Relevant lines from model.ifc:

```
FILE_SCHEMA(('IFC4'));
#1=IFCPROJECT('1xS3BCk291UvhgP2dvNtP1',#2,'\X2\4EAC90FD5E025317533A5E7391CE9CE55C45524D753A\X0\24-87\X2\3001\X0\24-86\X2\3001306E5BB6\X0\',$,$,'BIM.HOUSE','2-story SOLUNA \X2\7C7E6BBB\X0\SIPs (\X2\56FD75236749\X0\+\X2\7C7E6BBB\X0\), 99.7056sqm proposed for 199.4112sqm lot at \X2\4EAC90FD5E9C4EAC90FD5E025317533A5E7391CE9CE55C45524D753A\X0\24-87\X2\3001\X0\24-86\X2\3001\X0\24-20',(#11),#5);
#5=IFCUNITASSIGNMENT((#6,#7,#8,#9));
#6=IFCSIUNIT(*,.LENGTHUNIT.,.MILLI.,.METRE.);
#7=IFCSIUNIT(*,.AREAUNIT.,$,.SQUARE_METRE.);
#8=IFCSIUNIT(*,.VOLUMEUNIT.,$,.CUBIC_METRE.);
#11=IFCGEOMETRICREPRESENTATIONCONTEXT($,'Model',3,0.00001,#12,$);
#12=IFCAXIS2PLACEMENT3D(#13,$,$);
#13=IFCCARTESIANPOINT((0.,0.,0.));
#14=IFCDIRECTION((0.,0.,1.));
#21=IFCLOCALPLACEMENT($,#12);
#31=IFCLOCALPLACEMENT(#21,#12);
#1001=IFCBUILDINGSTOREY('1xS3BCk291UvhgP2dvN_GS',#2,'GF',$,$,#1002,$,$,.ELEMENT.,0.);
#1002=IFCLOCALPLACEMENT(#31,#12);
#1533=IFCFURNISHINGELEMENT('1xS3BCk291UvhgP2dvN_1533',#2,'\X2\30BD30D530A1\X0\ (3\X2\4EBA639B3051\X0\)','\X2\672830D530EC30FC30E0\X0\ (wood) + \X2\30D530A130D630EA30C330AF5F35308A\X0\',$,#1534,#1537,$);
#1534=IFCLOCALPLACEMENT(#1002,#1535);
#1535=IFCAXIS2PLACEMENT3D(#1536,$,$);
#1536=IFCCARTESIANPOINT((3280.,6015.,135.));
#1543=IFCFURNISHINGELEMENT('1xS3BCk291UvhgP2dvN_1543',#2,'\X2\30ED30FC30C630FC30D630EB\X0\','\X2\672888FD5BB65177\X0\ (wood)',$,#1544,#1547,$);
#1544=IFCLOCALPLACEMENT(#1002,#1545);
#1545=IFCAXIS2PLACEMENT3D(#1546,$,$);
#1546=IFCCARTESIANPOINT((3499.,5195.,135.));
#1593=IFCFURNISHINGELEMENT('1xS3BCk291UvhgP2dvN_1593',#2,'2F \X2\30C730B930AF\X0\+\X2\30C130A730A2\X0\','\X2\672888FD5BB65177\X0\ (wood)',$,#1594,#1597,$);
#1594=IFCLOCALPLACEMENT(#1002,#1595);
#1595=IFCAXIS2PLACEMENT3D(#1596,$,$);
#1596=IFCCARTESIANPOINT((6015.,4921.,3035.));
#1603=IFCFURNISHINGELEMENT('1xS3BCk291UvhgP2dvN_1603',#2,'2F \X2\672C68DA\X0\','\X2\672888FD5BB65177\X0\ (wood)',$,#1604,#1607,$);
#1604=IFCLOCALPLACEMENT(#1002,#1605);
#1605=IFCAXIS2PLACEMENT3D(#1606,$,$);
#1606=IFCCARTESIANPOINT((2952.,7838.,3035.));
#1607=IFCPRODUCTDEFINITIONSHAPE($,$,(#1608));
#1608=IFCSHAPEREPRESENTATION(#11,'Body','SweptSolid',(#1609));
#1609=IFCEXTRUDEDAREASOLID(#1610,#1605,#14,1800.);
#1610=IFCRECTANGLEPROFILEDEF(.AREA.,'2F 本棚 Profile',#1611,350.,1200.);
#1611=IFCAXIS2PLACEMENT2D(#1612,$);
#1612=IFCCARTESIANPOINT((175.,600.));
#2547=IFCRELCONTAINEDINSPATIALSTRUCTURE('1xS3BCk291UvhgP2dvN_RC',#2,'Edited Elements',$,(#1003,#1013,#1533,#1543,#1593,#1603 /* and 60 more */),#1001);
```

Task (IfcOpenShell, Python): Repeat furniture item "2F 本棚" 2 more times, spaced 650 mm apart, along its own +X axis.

```python
import ifcopenshell
import ifcopenshell.api.geometry
import ifcopenshell.api.root
import ifcopenshell.util.element
import ifcopenshell.util.placement

model = ifcopenshell.open("model.ifc")


def reuse_history(source, copy):
    """copy_class also copies each property set's owner history, people and application; keep the originals."""
    for rel in copy.IsDefinedBy:
        if rel.is_a("IfcRelDefinesByProperties") and (history := rel.RelatingPropertyDefinition.OwnerHistory):
            rel.RelatingPropertyDefinition.OwnerHistory = source.OwnerHistory
            ifcopenshell.util.element.remove_deep2(model, history)


source = model.by_guid("1xS3BCk291UvhgP2dvN_1603")
base = ifcopenshell.util.placement.get_local_placement(source.ObjectPlacement)
step = base[:3, 0] * 650.0

for i in range(1, 3):
    copy = ifcopenshell.api.root.copy_class(model, product=source)
    copy.Representation = ifcopenshell.util.element.copy_deep(
        model, source.Representation, exclude=["IfcGeometricRepresentationContext", "IfcRepresentationMap"]
    )
    reuse_history(source, copy)
    matrix = base.copy()
    matrix[:3, 3] += i * step
    print("added at", matrix[:3, 3].round(3) + 0.0)
    ifcopenshell.api.geometry.edit_object_placement(model, product=copy, matrix=matrix, is_si=False)

model.write("model_edited.ifc")
```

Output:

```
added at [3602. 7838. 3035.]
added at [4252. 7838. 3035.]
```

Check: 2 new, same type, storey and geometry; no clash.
